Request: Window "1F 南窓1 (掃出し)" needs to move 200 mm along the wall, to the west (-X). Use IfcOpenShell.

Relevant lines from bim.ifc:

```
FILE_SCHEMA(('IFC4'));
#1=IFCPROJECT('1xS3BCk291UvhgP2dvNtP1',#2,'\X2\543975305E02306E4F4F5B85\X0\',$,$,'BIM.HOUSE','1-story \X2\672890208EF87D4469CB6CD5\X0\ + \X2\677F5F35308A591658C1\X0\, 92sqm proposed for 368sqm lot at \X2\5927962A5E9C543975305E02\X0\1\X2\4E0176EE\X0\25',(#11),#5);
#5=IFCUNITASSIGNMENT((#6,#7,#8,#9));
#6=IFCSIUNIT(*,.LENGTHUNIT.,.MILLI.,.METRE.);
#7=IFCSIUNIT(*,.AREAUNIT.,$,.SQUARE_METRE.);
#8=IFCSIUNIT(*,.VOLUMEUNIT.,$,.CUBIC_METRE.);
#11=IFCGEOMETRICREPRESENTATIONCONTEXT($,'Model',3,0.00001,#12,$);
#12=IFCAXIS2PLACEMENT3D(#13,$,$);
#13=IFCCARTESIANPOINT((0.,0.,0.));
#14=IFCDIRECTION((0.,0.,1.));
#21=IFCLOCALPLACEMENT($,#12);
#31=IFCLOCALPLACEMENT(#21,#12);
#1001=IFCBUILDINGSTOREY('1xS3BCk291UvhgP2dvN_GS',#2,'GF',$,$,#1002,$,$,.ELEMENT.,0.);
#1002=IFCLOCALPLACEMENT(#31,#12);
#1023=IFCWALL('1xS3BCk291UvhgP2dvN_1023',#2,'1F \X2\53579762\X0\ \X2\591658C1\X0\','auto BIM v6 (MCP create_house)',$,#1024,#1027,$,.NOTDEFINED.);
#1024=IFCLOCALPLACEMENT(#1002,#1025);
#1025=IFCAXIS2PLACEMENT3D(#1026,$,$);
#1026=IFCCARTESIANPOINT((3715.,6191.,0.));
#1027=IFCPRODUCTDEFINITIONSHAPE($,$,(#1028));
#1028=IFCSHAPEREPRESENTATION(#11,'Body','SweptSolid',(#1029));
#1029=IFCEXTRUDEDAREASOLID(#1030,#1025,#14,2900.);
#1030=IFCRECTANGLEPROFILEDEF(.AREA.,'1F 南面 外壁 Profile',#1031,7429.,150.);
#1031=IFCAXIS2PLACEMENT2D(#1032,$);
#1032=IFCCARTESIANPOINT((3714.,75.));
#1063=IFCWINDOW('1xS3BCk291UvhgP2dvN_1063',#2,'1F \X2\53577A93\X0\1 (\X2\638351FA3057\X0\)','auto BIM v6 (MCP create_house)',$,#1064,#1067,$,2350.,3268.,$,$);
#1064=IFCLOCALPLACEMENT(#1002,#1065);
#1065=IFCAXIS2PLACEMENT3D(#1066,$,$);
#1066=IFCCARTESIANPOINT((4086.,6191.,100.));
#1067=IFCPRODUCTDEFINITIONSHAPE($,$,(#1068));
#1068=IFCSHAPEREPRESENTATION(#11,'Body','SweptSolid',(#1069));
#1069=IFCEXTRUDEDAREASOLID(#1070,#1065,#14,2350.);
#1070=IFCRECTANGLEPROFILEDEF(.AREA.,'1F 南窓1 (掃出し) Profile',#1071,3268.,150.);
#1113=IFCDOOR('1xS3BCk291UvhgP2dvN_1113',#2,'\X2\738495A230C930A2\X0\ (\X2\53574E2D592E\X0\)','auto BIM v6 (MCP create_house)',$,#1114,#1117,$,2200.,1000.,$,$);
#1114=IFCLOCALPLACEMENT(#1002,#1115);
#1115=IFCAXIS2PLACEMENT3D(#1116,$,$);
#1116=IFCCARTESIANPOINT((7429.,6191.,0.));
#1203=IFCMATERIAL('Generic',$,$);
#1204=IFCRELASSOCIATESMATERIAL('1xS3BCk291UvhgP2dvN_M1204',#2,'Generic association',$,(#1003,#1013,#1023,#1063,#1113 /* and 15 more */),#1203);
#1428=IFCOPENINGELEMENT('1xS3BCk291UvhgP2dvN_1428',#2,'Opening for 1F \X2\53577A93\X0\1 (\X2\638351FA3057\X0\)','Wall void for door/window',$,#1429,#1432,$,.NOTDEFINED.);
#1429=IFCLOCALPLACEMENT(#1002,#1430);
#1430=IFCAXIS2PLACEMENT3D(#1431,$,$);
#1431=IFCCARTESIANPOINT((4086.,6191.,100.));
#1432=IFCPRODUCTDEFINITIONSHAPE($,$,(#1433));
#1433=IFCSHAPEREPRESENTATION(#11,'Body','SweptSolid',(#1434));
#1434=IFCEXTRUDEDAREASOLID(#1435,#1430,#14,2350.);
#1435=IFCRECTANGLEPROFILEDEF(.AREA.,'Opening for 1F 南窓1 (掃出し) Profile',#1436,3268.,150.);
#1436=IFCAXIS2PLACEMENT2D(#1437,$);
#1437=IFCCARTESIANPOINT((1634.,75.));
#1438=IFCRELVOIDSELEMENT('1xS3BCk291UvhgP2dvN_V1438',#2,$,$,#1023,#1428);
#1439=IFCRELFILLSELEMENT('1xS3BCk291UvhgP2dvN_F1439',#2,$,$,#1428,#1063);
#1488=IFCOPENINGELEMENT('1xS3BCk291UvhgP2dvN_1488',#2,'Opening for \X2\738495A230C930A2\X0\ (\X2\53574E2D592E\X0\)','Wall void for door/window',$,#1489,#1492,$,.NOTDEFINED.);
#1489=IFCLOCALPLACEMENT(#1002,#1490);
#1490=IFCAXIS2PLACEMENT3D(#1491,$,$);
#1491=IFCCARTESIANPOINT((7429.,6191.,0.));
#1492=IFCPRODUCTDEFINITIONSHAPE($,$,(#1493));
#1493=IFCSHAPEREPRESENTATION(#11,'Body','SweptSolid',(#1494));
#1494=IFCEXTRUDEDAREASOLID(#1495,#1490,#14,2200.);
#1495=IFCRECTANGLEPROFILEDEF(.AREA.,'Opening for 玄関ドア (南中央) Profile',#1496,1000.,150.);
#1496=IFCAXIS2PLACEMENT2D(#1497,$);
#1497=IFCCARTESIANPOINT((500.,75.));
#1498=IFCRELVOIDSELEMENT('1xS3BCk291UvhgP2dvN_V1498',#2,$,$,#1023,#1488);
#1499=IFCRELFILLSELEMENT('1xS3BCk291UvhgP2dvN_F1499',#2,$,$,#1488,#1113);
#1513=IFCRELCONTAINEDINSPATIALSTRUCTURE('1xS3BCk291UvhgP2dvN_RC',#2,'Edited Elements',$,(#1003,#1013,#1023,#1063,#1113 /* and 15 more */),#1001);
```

```python
import ifcopenshell
import ifcopenshell.api.geometry
import ifcopenshell.util.placement
import ifcopenshell.util.unit

model = ifcopenshell.open("bim.ifc")
unit_scale = ifcopenshell.util.unit.calculate_unit_scale(model)

window = model.by_guid("1xS3BCk291UvhgP2dvN_1063")
opening = window.FillsVoids[0].RelatingOpeningElement
wall = opening.VoidsElements[0].RelatingBuildingElement

wall_matrix = ifcopenshell.util.placement.get_local_placement(wall.ObjectPlacement)
shift = wall_matrix[:3, 0] * -0.2 / unit_scale
before = ifcopenshell.util.placement.get_local_placement(window.ObjectPlacement)[:3, 3].copy()

# The window is not placed relative to its opening, so move both.
for product in (opening, window):
    matrix = ifcopenshell.util.placement.get_local_placement(product.ObjectPlacement)
    matrix[:3, 3] += shift
    ifcopenshell.api.geometry.edit_object_placement(model, product=product, matrix=matrix, is_si=False)

after = ifcopenshell.util.placement.get_local_placement(window.ObjectPlacement)[:3, 3]
print("window moved by", (after - before).round(3) + 0.0)

model.write("bim-out.ifc")
```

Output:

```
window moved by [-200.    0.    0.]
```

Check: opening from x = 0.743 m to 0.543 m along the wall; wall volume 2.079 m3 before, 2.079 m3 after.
